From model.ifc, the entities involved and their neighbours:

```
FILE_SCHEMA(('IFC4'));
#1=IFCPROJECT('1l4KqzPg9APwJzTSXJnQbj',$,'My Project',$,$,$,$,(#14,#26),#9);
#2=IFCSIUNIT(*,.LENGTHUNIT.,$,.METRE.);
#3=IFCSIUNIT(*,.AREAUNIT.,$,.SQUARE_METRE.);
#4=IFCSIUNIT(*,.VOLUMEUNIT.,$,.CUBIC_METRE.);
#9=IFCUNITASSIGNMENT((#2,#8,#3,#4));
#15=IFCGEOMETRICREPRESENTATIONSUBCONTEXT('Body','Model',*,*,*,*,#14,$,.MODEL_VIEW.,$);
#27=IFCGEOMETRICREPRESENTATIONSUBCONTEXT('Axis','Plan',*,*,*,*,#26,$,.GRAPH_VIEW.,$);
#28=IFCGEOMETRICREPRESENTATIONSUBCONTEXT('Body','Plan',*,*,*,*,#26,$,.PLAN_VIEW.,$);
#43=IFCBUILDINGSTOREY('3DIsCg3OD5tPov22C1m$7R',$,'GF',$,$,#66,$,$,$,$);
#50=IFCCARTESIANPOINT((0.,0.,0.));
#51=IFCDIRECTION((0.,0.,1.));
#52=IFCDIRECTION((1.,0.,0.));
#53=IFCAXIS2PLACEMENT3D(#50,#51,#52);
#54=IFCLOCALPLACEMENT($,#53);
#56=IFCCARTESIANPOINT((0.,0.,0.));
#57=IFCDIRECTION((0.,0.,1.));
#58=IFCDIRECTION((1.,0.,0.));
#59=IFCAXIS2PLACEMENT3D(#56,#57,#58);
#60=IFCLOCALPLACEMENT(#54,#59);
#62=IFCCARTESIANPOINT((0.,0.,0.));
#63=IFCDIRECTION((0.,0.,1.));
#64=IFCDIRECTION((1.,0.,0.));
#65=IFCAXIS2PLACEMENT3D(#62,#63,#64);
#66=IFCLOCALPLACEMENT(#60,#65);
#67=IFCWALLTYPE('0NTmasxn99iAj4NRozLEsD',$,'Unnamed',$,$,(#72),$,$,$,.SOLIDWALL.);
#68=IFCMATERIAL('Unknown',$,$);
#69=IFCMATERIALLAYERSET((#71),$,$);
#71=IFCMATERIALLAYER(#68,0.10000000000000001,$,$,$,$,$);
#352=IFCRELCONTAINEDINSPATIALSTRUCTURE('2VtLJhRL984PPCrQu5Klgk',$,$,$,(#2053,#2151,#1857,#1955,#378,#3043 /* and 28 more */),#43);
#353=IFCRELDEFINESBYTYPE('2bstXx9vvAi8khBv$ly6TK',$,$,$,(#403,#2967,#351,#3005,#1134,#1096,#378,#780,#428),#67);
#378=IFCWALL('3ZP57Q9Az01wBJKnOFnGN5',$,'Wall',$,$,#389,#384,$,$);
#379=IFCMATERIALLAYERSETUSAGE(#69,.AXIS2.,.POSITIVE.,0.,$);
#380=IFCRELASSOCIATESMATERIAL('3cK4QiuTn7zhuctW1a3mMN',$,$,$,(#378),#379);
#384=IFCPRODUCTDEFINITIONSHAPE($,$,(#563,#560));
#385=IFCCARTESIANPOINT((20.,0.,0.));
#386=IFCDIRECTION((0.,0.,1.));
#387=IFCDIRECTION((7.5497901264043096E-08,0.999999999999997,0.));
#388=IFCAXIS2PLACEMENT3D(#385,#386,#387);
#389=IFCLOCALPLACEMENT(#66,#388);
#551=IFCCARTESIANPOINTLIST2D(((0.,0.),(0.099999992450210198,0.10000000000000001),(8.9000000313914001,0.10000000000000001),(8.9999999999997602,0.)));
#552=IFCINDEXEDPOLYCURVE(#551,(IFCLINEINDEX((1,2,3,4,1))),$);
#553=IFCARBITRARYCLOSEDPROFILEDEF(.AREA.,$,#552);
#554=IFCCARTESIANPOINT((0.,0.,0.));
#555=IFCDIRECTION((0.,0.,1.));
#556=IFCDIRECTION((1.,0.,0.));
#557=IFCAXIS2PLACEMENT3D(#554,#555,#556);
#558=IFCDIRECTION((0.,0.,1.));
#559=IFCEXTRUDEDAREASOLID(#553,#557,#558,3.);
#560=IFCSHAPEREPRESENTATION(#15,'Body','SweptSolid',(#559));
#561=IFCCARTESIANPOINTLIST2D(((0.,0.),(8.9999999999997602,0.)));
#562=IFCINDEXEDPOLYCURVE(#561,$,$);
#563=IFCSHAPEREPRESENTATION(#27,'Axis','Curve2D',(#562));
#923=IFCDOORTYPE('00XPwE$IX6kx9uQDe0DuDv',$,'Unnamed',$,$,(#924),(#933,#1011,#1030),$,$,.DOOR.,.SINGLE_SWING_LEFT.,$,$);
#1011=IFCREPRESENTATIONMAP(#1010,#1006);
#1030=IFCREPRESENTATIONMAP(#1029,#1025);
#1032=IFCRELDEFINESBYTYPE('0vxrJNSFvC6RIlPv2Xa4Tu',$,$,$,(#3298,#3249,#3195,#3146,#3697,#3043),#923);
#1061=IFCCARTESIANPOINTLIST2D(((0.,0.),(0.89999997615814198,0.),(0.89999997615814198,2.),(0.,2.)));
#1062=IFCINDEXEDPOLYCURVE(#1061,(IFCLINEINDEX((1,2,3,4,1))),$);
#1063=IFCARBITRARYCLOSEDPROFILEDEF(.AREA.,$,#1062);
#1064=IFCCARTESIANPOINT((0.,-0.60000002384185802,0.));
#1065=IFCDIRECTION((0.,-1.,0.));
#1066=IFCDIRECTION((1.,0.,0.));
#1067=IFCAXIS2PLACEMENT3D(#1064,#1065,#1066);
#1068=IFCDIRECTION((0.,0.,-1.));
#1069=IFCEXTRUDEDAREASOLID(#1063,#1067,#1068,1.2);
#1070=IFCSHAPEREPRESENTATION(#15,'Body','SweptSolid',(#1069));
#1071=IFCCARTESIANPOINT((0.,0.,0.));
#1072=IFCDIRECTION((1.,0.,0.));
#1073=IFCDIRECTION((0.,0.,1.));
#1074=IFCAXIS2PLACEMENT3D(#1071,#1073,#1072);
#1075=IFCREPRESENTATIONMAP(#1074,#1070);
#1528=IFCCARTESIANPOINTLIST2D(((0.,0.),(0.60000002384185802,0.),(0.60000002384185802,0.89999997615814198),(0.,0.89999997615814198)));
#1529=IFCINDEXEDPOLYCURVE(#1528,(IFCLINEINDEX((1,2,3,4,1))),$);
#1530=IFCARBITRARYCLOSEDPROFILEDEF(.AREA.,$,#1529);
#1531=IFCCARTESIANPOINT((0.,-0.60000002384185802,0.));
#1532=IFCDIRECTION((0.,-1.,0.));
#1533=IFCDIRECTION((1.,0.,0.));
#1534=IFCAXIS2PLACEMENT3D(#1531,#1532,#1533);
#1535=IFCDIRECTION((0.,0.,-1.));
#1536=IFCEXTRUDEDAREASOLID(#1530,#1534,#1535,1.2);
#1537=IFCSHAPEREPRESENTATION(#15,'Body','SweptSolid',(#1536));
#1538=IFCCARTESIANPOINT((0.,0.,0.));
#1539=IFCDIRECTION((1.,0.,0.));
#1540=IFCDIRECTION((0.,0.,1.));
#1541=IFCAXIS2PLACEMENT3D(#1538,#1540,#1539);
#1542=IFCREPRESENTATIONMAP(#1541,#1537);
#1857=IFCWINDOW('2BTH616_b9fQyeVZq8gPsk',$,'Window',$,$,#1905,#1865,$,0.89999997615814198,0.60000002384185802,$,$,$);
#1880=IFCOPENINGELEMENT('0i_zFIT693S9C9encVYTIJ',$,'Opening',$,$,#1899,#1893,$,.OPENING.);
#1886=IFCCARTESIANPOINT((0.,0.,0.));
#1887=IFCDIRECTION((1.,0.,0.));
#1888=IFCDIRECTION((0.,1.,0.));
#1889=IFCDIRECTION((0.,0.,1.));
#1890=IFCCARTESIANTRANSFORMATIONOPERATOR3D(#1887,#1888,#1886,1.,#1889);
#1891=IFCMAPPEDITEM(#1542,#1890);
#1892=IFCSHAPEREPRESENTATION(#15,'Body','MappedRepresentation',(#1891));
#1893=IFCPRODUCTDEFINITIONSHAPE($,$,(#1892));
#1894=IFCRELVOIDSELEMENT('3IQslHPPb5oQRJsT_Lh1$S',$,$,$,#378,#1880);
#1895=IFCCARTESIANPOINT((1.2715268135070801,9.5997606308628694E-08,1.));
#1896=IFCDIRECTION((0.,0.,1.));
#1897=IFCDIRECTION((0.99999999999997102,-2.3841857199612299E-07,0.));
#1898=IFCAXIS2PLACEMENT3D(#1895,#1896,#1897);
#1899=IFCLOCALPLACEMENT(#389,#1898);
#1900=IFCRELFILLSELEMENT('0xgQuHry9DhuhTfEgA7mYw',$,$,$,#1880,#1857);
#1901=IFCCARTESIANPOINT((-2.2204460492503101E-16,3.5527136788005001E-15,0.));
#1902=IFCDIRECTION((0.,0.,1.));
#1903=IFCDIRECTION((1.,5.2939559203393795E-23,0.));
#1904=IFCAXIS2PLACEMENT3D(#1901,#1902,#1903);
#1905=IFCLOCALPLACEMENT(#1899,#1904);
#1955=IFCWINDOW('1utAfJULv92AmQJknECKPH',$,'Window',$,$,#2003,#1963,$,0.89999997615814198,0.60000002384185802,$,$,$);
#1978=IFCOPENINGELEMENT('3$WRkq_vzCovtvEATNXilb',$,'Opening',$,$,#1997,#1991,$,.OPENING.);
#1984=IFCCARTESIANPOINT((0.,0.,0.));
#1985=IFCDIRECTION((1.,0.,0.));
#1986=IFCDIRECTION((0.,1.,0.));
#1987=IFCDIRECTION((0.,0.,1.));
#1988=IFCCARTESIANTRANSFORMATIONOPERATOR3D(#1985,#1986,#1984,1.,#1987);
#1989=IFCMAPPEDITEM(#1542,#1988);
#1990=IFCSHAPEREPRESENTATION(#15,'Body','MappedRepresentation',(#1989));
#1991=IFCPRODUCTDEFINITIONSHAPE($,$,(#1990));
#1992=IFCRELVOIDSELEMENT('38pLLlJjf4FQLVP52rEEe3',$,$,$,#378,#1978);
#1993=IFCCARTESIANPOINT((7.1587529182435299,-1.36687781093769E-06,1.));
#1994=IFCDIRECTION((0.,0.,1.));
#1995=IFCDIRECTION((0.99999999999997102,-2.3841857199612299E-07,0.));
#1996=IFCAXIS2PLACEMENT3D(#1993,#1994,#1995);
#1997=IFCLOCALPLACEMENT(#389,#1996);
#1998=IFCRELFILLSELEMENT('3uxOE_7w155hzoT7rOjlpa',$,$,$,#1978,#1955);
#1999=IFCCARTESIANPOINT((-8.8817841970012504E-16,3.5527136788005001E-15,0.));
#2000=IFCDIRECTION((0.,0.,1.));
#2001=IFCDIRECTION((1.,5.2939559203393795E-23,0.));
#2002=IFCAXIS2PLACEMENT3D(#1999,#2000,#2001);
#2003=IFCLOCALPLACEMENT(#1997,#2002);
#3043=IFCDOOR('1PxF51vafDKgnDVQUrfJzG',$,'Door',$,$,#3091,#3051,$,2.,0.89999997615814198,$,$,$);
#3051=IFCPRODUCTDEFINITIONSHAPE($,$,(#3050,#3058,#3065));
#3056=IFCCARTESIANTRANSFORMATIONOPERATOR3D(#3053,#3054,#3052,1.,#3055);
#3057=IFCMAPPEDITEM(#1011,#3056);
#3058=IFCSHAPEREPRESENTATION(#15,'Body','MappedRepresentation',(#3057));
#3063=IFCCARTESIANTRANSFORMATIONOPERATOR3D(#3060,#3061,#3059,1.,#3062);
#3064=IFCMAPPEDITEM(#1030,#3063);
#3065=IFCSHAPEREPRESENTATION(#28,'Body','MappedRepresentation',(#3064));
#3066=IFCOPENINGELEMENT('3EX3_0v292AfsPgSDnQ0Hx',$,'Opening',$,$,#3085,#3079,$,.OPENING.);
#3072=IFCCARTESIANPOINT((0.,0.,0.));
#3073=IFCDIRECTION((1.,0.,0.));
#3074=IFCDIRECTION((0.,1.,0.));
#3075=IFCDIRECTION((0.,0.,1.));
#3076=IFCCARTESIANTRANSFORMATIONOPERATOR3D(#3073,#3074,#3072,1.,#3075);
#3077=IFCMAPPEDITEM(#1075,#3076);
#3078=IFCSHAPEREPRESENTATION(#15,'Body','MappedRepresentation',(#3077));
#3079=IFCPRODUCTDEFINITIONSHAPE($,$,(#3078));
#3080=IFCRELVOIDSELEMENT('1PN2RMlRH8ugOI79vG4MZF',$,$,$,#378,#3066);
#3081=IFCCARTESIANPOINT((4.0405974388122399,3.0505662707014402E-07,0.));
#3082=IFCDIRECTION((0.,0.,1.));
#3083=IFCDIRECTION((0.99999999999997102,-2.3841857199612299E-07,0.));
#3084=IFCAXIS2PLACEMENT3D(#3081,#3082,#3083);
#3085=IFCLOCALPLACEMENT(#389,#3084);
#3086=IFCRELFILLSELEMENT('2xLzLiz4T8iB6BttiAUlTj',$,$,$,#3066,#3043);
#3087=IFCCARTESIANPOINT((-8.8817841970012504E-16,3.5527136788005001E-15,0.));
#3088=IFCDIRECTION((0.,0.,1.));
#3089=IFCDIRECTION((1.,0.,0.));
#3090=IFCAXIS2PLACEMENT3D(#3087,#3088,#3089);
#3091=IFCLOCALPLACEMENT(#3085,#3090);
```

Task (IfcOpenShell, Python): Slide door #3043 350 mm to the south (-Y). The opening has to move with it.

```python
import ifcopenshell
import ifcopenshell.api.geometry
import ifcopenshell.util.placement
import ifcopenshell.util.unit

model = ifcopenshell.open("model.ifc")
unit_scale = ifcopenshell.util.unit.calculate_unit_scale(model)

door = model.by_guid("1PxF51vafDKgnDVQUrfJzG")
opening = door.FillsVoids[0].RelatingOpeningElement
wall = opening.VoidsElements[0].RelatingBuildingElement

wall_matrix = ifcopenshell.util.placement.get_local_placement(wall.ObjectPlacement)
shift = wall_matrix[:3, 0] * -0.35 / unit_scale
before = ifcopenshell.util.placement.get_local_placement(door.ObjectPlacement)[:3, 3].copy()

# The door is placed relative to its opening, so it follows when the opening moves.
matrix = ifcopenshell.util.placement.get_local_placement(opening.ObjectPlacement)
matrix[:3, 3] += shift
ifcopenshell.api.geometry.edit_object_placement(
    model, product=opening, matrix=matrix, is_si=False, should_transform_children=True
)

after = ifcopenshell.util.placement.get_local_placement(door.ObjectPlacement)[:3, 3]
print("door moved by", (after - before).round(3) + 0.0)

model.write("model_rev.ifc")
```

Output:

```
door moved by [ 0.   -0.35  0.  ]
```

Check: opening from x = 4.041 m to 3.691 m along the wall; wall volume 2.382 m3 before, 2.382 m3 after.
